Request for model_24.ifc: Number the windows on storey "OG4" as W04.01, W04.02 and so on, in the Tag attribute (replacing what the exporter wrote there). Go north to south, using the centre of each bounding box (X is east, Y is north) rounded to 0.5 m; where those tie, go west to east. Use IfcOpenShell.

First a look at what the model holds.

```python
import ifcopenshell
import ifcopenshell.util.element
import ifcopenshell.util.placement

model = ifcopenshell.open("model_24.ifc")
print(model.schema)
storey = next(s for s in model.by_type("IfcBuildingStorey") if s.Name == "OG4")
windows = [e for e in ifcopenshell.util.element.get_decomposition(storey) if e.is_a("IfcWindow")]
for e in sorted(windows, key=lambda e: e.id()):
    origin = ifcopenshell.util.placement.get_local_placement(e.ObjectPlacement)[:3, 3]
    print(e.id(), e.Tag, e.Name, origin.round(2) + 0.0, sep=" | ")
```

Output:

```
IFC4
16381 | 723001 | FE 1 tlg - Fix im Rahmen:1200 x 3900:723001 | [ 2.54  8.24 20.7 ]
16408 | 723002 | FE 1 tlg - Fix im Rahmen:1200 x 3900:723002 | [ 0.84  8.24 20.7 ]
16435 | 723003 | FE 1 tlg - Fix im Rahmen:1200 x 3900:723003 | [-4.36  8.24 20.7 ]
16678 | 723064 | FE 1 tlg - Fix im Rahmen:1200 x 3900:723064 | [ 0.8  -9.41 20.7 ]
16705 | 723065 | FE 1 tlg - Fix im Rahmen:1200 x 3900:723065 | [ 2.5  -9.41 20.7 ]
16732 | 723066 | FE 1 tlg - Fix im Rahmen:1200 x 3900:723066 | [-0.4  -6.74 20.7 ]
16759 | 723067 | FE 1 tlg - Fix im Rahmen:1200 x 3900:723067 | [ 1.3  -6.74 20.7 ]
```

```python
import ifcopenshell
import ifcopenshell.geom
import ifcopenshell.util.element
import ifcopenshell.util.shape

model = ifcopenshell.open("model_24.ifc")
settings = ifcopenshell.geom.settings()
settings.set("use-world-coords", True)


def centre(element):
    shape = ifcopenshell.geom.create_shape(settings, element)
    return ifcopenshell.util.shape.get_bbox_centroid(shape.geometry)


storey = next(s for s in model.by_type("IfcBuildingStorey") if s.Name == "OG4")
windows = [e for e in ifcopenshell.util.element.get_decomposition(storey) if e.is_a("IfcWindow")]

# Insertion points can sit at a corner or the storey origin, so sort by the geometry (in metres).
centres = {e: centre(e) for e in windows}
windows.sort(key=lambda e: (-round(centres[e][1] / 0.5), centres[e][0]))

for i, e in enumerate(windows, start=1):
    number = f"W04.{i:02d}"
    e.Tag = number
    print(e.id(), number)

model.write("model_24_rev.ifc")
```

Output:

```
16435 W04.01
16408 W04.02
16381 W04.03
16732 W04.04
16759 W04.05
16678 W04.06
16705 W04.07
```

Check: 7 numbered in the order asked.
